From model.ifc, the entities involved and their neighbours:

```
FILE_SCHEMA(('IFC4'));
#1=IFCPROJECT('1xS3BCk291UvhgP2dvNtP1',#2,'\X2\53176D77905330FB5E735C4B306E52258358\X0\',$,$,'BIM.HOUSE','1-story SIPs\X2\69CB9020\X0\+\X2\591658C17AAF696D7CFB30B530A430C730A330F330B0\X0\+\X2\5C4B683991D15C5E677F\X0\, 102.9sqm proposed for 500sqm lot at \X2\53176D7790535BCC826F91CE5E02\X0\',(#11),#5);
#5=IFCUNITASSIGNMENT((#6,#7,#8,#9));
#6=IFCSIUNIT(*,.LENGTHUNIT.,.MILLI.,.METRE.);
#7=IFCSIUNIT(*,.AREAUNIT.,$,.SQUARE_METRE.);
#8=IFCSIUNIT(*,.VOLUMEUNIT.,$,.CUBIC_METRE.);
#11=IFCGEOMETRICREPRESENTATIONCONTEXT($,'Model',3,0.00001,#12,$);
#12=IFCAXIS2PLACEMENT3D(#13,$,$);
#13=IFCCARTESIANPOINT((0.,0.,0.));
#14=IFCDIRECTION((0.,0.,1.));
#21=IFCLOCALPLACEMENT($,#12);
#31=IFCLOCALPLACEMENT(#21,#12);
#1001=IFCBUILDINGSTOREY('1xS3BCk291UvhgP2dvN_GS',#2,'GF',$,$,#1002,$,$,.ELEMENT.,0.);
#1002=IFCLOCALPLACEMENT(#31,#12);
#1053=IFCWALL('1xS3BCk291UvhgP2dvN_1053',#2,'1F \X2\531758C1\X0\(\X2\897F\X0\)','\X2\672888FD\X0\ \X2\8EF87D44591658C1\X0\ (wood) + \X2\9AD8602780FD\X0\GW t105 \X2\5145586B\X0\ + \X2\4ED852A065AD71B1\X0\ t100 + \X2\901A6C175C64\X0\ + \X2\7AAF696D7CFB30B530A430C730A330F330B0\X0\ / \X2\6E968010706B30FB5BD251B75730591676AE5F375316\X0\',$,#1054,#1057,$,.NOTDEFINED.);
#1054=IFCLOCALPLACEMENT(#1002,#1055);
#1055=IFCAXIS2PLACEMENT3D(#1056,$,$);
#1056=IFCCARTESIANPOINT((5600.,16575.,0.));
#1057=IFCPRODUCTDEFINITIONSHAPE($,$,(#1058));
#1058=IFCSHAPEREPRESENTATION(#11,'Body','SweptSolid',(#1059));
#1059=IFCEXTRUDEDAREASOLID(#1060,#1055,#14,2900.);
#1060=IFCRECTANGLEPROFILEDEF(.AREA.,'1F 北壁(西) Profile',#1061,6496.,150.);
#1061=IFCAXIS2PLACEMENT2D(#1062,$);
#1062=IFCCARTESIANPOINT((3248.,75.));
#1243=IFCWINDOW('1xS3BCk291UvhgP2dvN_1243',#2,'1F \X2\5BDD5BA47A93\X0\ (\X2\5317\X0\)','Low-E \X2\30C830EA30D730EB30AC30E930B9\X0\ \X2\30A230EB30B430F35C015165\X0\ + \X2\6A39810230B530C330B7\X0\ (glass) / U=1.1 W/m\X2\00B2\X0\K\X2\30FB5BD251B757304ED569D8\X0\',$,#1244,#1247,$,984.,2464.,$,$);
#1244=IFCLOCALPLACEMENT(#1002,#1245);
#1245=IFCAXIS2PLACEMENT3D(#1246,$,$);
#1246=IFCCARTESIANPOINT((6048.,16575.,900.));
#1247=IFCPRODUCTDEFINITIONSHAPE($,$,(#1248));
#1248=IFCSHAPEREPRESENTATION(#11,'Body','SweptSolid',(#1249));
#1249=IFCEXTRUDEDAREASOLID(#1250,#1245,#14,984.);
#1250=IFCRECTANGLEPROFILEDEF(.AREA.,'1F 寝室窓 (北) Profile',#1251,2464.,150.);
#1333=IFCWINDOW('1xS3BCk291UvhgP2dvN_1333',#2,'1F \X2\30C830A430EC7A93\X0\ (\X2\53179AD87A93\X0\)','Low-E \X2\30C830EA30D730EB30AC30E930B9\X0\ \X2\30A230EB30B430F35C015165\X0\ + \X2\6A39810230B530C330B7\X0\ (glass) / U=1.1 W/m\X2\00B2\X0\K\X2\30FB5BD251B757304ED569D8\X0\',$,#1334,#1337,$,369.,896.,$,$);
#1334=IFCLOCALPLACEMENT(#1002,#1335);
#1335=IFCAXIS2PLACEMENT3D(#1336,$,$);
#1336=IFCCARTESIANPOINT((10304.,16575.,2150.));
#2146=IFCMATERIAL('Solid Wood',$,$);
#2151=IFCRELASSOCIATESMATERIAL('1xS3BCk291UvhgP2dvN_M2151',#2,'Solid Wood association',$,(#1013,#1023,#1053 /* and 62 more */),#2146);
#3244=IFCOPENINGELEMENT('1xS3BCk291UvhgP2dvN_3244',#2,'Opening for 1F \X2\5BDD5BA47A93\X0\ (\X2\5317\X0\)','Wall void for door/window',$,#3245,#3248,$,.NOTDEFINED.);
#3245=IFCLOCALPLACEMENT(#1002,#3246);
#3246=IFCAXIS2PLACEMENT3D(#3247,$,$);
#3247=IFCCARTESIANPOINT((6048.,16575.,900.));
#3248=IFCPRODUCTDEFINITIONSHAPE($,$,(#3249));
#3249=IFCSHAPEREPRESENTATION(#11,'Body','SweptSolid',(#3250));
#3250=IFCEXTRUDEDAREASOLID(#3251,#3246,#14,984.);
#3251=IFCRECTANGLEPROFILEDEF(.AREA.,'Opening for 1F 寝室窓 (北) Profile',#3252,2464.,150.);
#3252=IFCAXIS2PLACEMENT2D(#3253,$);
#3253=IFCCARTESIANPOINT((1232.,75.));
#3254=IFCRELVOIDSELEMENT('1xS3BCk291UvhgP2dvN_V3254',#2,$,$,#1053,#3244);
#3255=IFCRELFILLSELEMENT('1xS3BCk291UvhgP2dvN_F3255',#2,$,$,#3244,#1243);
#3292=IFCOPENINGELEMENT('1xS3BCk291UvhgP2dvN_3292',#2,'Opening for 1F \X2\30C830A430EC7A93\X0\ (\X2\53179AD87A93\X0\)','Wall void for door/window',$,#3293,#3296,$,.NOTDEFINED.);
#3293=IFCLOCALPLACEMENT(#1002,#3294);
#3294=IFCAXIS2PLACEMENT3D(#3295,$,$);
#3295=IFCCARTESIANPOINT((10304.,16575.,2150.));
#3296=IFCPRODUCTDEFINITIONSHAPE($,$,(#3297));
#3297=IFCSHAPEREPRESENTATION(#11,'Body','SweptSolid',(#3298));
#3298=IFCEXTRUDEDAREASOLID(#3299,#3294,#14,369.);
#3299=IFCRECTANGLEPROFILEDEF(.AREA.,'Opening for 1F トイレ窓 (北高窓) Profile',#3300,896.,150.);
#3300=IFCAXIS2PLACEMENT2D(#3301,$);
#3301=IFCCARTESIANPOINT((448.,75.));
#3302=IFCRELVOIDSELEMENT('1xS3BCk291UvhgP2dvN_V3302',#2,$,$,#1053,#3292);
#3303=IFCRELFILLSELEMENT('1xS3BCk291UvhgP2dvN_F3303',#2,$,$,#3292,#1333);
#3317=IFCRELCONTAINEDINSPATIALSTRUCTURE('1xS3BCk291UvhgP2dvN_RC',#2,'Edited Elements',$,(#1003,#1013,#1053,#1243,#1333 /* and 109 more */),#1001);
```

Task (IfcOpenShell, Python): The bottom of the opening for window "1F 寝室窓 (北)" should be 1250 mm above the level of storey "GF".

```python
import numpy as np
import ifcopenshell
import ifcopenshell.api.geometry
import ifcopenshell.geom
import ifcopenshell.util.element
import ifcopenshell.util.placement
import ifcopenshell.util.shape
import ifcopenshell.util.unit

model = ifcopenshell.open("model.ifc")
unit_scale = ifcopenshell.util.unit.calculate_unit_scale(model)

window = model.by_guid("1xS3BCk291UvhgP2dvN_1243")
opening = window.FillsVoids[0].RelatingOpeningElement
storey = ifcopenshell.util.element.get_container(window, ifc_class="IfcBuildingStorey")
level = ifcopenshell.util.placement.get_local_placement(storey.ObjectPlacement)[2, 3]

# The opening's origin need not be at the sill, so measure its lowest point.
shape = ifcopenshell.geom.create_shape(ifcopenshell.geom.settings(), opening)
bottom = ifcopenshell.util.shape.get_shape_bottom_elevation(shape, shape.geometry) / unit_scale
dz = level + 1.25 / unit_scale - bottom

shift = np.array([0.0, 0.0, dz])
# The window is not placed relative to its opening, so move both.
for product in (opening, window):
    matrix = ifcopenshell.util.placement.get_local_placement(product.ObjectPlacement)
    matrix[:3, 3] += shift
    ifcopenshell.api.geometry.edit_object_placement(model, product=product, matrix=matrix, is_si=False)

print(f"moved by {dz * unit_scale:+.3f} m")

model.write("model_v2.ifc")
```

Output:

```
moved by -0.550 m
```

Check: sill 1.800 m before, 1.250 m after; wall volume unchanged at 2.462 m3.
